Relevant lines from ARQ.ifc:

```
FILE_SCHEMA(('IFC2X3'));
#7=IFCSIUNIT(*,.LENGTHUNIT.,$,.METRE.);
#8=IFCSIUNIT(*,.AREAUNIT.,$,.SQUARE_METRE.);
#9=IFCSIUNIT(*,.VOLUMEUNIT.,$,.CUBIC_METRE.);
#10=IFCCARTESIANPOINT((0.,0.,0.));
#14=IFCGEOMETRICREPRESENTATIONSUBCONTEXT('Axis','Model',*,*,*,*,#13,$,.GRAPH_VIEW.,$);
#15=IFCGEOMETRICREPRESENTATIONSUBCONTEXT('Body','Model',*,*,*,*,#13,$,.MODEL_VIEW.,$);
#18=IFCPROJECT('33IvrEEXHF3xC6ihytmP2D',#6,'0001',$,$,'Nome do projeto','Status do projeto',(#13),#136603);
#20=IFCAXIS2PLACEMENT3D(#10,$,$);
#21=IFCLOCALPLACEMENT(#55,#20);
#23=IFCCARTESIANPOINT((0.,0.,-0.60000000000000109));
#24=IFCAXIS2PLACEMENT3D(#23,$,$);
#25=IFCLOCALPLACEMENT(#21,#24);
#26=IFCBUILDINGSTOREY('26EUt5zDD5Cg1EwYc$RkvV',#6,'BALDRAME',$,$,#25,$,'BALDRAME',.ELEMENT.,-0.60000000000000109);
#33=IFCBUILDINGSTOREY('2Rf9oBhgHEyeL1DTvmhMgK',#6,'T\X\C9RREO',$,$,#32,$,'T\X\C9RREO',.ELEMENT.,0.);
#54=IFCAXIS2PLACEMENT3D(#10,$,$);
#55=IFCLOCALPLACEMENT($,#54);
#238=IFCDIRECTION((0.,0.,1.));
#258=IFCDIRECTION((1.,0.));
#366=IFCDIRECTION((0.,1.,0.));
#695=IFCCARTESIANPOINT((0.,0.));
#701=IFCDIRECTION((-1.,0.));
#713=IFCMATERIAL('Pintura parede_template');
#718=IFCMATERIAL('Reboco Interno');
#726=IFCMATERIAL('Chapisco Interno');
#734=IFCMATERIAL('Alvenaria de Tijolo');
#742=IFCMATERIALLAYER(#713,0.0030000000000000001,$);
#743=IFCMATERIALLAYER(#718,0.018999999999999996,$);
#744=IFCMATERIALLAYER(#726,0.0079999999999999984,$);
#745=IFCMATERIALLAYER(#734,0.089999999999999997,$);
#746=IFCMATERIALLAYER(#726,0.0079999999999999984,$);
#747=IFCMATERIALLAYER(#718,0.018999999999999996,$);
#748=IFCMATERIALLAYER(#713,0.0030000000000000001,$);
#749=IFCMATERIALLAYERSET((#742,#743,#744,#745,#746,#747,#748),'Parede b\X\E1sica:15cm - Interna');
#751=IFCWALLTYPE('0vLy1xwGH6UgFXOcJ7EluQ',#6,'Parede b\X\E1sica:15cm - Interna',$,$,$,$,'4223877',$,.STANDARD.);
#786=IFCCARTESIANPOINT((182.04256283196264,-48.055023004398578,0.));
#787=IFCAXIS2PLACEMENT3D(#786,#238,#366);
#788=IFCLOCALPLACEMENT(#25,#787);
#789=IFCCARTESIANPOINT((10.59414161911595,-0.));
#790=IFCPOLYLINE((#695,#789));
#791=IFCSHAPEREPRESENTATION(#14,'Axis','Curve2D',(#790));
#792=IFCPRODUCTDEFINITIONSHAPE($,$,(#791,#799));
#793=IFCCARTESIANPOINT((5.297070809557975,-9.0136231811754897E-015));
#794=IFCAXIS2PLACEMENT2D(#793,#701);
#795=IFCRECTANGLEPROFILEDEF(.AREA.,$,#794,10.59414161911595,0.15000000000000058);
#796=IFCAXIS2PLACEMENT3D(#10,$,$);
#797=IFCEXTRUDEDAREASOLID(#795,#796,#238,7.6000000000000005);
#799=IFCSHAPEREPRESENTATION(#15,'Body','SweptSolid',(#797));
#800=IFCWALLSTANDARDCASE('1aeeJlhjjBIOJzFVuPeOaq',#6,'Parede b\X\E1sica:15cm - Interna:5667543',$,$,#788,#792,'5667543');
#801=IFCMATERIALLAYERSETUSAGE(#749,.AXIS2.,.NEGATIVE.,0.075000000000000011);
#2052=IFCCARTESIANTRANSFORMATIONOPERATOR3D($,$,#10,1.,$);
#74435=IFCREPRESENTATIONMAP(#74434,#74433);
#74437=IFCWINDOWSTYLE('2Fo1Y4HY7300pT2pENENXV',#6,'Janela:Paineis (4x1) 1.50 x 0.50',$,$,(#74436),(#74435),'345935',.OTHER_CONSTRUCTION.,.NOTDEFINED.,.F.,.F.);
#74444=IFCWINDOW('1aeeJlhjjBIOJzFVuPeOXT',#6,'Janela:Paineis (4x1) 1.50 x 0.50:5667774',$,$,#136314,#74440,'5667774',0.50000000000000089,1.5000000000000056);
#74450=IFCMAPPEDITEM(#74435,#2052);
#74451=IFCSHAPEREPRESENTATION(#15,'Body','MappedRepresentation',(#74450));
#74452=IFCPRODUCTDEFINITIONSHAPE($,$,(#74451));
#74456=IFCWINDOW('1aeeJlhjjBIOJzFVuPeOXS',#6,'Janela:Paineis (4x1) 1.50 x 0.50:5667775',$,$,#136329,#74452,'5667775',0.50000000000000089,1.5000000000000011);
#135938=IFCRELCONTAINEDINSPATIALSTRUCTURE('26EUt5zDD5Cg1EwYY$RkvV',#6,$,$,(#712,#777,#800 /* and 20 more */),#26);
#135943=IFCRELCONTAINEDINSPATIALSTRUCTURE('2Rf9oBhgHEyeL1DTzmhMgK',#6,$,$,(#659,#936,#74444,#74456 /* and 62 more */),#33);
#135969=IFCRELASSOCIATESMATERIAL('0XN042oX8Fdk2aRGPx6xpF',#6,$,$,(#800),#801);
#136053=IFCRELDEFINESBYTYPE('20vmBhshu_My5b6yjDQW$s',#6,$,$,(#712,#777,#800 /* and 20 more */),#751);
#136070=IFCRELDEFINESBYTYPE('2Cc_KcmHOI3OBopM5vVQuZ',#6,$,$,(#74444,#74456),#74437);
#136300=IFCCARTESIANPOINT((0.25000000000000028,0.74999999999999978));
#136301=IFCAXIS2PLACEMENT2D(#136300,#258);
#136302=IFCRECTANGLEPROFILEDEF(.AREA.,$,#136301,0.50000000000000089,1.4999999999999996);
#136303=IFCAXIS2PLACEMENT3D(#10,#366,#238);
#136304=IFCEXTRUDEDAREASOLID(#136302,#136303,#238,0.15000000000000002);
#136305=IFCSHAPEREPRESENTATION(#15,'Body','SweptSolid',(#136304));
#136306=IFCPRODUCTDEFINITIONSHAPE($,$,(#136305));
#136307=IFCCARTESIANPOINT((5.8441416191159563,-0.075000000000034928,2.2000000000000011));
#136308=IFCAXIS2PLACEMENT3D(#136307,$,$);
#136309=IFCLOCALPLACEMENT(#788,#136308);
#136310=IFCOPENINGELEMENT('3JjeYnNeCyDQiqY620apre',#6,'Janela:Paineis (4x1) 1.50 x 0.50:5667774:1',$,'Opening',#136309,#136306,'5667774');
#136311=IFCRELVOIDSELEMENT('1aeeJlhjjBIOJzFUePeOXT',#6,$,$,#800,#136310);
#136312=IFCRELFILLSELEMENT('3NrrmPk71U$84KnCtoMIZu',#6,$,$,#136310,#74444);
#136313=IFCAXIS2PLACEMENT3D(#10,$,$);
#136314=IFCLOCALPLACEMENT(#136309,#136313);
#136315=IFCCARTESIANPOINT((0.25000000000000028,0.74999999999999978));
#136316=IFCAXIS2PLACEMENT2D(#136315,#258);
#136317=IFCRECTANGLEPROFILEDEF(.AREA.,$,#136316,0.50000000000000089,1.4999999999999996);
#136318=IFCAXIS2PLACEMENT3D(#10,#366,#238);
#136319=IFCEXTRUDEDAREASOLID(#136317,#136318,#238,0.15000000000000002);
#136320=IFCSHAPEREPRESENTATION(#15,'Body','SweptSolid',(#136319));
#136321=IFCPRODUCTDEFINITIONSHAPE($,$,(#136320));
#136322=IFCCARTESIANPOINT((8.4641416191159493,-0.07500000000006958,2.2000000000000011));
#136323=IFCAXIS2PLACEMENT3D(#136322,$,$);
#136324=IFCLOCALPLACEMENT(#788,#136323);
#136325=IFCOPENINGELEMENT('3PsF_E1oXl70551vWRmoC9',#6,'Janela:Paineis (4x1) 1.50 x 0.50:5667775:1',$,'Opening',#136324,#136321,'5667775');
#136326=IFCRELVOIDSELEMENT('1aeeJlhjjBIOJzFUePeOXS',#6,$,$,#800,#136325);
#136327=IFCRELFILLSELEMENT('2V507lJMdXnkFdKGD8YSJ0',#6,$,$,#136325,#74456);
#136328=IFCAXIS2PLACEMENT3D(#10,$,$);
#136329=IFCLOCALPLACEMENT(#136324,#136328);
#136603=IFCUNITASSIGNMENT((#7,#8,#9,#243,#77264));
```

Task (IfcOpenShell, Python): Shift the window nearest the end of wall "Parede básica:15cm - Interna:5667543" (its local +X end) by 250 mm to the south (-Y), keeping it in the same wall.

```python
import ifcopenshell
import ifcopenshell.api.geometry
import ifcopenshell.util.placement
import ifcopenshell.util.unit

model = ifcopenshell.open("ARQ.ifc")
unit_scale = ifcopenshell.util.unit.calculate_unit_scale(model)

window = model.by_guid("1aeeJlhjjBIOJzFVuPeOXS")
opening = window.FillsVoids[0].RelatingOpeningElement
wall = opening.VoidsElements[0].RelatingBuildingElement

wall_matrix = ifcopenshell.util.placement.get_local_placement(wall.ObjectPlacement)
shift = wall_matrix[:3, 0] * -0.25 / unit_scale
before = ifcopenshell.util.placement.get_local_placement(window.ObjectPlacement)[:3, 3].copy()

# The window is placed relative to its opening, so it follows when the opening moves.
matrix = ifcopenshell.util.placement.get_local_placement(opening.ObjectPlacement)
matrix[:3, 3] += shift
ifcopenshell.api.geometry.edit_object_placement(
    model, product=opening, matrix=matrix, is_si=False, should_transform_children=True
)

after = ifcopenshell.util.placement.get_local_placement(window.ObjectPlacement)[:3, 3]
print("window moved by", (after - before).round(3) + 0.0)

model.write("ARQ_rev.ifc")
```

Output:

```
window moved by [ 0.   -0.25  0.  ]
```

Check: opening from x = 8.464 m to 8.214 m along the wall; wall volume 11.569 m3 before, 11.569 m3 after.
